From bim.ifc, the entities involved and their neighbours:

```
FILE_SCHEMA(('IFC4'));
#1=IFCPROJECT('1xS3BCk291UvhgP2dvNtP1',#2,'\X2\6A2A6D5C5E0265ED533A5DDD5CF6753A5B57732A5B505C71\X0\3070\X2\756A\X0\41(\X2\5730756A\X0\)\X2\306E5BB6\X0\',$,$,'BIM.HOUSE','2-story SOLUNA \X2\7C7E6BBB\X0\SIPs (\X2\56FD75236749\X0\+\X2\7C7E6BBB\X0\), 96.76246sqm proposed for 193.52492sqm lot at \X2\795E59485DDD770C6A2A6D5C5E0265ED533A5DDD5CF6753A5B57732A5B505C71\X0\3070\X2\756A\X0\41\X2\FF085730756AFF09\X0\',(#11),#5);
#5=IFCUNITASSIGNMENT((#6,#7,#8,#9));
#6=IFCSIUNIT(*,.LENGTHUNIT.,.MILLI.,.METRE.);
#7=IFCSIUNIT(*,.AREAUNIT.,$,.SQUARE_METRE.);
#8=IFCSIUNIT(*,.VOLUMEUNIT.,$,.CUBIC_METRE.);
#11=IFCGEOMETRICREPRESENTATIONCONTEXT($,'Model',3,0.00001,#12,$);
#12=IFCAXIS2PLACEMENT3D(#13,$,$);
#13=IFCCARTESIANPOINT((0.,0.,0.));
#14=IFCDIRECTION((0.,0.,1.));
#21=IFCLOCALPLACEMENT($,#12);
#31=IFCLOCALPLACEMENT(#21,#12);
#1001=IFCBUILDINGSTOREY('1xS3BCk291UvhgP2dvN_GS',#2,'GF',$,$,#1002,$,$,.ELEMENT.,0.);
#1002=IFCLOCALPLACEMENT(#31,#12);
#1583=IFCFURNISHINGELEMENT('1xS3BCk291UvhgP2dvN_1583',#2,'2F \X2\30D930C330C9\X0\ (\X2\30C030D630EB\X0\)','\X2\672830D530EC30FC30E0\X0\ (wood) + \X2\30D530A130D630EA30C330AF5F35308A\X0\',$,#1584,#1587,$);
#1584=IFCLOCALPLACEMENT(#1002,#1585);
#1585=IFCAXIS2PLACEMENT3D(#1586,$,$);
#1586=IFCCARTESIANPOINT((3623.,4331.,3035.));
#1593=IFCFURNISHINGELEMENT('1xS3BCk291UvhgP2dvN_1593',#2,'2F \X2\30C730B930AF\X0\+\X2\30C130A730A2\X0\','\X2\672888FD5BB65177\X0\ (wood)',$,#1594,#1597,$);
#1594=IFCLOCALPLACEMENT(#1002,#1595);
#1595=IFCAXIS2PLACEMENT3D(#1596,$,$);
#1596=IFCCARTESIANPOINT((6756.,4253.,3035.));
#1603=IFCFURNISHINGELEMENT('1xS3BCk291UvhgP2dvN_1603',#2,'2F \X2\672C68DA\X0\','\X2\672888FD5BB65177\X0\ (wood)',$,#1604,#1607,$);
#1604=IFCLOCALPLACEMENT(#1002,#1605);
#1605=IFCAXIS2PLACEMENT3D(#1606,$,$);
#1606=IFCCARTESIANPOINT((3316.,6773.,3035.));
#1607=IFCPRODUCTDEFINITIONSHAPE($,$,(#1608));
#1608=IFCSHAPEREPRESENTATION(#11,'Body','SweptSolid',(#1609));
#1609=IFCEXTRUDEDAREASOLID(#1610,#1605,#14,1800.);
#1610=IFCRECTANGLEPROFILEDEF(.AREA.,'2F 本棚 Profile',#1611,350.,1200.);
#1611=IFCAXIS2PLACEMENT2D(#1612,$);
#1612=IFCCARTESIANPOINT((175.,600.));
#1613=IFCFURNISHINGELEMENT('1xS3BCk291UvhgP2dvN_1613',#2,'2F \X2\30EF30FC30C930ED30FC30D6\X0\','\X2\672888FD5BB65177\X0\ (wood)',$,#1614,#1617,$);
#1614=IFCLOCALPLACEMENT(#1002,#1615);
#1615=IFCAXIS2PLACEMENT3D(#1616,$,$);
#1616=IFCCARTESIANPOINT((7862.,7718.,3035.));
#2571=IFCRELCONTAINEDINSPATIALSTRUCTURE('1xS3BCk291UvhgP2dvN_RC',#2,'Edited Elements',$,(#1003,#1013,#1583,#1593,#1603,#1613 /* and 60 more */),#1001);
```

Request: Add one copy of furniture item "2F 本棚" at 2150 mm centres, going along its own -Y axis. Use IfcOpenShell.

```python
import ifcopenshell
import ifcopenshell.api.geometry
import ifcopenshell.api.root
import ifcopenshell.util.element
import ifcopenshell.util.placement
import ifcopenshell.util.unit

model = ifcopenshell.open("bim.ifc")
unit_scale = ifcopenshell.util.unit.calculate_unit_scale(model)


def reuse_history(source, copy):
    """copy_class also copies each property set's owner history, people and application; keep the originals."""
    for rel in copy.IsDefinedBy:
        if rel.is_a("IfcRelDefinesByProperties") and (history := rel.RelatingPropertyDefinition.OwnerHistory):
            rel.RelatingPropertyDefinition.OwnerHistory = source.OwnerHistory
            ifcopenshell.util.element.remove_deep2(model, history)


source = model.by_guid("1xS3BCk291UvhgP2dvN_1603")
base = ifcopenshell.util.placement.get_local_placement(source.ObjectPlacement)
step = -base[:3, 1] * 2.15 / unit_scale

for i in range(1, 2):
    copy = ifcopenshell.api.root.copy_class(model, product=source)
    copy.Representation = ifcopenshell.util.element.copy_deep(
        model, source.Representation, exclude=["IfcGeometricRepresentationContext", "IfcRepresentationMap"]
    )
    reuse_history(source, copy)
    matrix = base.copy()
    matrix[:3, 3] += i * step
    print("added at", matrix[:3, 3].round(3) + 0.0)
    ifcopenshell.api.geometry.edit_object_placement(model, product=copy, matrix=matrix, is_si=False)

model.write("bim_edited.ifc")
```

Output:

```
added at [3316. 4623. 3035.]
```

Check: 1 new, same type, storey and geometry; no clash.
